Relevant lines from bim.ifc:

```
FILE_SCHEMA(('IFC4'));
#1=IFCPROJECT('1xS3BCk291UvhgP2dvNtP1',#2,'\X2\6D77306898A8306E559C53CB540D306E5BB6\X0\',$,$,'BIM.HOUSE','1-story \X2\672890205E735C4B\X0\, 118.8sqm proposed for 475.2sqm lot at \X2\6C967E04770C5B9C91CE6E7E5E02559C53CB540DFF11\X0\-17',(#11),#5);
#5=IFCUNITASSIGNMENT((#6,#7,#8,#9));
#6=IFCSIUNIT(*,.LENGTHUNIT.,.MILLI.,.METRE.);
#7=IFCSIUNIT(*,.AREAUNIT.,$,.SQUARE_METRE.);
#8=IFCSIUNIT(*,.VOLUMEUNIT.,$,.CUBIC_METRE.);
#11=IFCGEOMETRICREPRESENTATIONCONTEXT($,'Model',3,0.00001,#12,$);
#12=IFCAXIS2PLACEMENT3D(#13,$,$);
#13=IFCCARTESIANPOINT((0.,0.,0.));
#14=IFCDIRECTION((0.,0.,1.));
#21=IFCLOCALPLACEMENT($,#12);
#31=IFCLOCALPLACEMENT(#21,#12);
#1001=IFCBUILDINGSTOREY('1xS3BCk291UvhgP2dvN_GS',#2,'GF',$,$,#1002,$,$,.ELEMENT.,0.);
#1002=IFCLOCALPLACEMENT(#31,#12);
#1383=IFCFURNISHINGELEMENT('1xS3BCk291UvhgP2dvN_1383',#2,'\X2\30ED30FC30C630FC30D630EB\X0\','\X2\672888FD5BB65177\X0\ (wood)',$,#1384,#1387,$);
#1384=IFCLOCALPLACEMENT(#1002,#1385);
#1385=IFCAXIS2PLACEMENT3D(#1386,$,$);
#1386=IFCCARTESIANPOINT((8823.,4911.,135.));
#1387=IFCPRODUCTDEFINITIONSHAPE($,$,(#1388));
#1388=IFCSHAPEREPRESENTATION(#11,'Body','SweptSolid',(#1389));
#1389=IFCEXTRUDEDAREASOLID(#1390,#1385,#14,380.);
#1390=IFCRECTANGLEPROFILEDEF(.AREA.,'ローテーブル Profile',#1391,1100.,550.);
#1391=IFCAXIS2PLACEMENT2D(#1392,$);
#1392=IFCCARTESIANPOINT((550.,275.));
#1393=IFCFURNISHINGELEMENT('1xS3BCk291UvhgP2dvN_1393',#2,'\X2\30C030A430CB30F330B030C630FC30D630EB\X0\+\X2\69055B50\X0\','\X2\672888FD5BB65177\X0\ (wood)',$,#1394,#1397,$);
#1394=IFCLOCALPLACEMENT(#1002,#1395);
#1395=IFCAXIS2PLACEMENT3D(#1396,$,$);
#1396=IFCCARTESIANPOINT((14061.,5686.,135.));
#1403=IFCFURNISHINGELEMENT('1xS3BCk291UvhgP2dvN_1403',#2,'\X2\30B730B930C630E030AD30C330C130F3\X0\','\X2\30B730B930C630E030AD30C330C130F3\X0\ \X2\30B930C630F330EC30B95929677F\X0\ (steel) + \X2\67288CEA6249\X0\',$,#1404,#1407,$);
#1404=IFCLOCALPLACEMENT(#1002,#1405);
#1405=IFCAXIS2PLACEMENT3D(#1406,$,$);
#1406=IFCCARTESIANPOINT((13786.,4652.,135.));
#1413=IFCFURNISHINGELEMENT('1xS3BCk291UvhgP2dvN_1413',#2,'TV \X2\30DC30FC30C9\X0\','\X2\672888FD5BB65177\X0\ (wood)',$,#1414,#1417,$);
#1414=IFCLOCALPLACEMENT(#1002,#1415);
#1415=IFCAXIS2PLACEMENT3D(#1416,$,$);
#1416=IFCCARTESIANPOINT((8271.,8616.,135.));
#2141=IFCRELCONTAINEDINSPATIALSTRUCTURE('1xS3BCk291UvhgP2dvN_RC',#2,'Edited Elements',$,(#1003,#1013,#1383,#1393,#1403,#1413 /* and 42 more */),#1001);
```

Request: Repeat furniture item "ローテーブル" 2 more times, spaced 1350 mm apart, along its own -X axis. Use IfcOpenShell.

```python
import ifcopenshell
import ifcopenshell.api.geometry
import ifcopenshell.api.root
import ifcopenshell.util.element
import ifcopenshell.util.placement
import ifcopenshell.util.unit

model = ifcopenshell.open("bim.ifc")
unit_scale = ifcopenshell.util.unit.calculate_unit_scale(model)


def reuse_history(source, copy):
    """copy_class also copies each property set's owner history, people and application; keep the originals."""
    for rel in copy.IsDefinedBy:
        if rel.is_a("IfcRelDefinesByProperties") and (history := rel.RelatingPropertyDefinition.OwnerHistory):
            rel.RelatingPropertyDefinition.OwnerHistory = source.OwnerHistory
            ifcopenshell.util.element.remove_deep2(model, history)


source = model.by_guid("1xS3BCk291UvhgP2dvN_1383")
base = ifcopenshell.util.placement.get_local_placement(source.ObjectPlacement)
step = -base[:3, 0] * 1.35 / unit_scale

for i in range(1, 3):
    copy = ifcopenshell.api.root.copy_class(model, product=source)
    copy.Representation = ifcopenshell.util.element.copy_deep(
        model, source.Representation, exclude=["IfcGeometricRepresentationContext", "IfcRepresentationMap"]
    )
    reuse_history(source, copy)
    matrix = base.copy()
    matrix[:3, 3] += i * step
    print("added at", matrix[:3, 3].round(3) + 0.0)
    ifcopenshell.api.geometry.edit_object_placement(model, product=copy, matrix=matrix, is_si=False)

model.write("bim_rev.ifc")
```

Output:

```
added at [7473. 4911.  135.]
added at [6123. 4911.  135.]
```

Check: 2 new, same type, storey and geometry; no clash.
